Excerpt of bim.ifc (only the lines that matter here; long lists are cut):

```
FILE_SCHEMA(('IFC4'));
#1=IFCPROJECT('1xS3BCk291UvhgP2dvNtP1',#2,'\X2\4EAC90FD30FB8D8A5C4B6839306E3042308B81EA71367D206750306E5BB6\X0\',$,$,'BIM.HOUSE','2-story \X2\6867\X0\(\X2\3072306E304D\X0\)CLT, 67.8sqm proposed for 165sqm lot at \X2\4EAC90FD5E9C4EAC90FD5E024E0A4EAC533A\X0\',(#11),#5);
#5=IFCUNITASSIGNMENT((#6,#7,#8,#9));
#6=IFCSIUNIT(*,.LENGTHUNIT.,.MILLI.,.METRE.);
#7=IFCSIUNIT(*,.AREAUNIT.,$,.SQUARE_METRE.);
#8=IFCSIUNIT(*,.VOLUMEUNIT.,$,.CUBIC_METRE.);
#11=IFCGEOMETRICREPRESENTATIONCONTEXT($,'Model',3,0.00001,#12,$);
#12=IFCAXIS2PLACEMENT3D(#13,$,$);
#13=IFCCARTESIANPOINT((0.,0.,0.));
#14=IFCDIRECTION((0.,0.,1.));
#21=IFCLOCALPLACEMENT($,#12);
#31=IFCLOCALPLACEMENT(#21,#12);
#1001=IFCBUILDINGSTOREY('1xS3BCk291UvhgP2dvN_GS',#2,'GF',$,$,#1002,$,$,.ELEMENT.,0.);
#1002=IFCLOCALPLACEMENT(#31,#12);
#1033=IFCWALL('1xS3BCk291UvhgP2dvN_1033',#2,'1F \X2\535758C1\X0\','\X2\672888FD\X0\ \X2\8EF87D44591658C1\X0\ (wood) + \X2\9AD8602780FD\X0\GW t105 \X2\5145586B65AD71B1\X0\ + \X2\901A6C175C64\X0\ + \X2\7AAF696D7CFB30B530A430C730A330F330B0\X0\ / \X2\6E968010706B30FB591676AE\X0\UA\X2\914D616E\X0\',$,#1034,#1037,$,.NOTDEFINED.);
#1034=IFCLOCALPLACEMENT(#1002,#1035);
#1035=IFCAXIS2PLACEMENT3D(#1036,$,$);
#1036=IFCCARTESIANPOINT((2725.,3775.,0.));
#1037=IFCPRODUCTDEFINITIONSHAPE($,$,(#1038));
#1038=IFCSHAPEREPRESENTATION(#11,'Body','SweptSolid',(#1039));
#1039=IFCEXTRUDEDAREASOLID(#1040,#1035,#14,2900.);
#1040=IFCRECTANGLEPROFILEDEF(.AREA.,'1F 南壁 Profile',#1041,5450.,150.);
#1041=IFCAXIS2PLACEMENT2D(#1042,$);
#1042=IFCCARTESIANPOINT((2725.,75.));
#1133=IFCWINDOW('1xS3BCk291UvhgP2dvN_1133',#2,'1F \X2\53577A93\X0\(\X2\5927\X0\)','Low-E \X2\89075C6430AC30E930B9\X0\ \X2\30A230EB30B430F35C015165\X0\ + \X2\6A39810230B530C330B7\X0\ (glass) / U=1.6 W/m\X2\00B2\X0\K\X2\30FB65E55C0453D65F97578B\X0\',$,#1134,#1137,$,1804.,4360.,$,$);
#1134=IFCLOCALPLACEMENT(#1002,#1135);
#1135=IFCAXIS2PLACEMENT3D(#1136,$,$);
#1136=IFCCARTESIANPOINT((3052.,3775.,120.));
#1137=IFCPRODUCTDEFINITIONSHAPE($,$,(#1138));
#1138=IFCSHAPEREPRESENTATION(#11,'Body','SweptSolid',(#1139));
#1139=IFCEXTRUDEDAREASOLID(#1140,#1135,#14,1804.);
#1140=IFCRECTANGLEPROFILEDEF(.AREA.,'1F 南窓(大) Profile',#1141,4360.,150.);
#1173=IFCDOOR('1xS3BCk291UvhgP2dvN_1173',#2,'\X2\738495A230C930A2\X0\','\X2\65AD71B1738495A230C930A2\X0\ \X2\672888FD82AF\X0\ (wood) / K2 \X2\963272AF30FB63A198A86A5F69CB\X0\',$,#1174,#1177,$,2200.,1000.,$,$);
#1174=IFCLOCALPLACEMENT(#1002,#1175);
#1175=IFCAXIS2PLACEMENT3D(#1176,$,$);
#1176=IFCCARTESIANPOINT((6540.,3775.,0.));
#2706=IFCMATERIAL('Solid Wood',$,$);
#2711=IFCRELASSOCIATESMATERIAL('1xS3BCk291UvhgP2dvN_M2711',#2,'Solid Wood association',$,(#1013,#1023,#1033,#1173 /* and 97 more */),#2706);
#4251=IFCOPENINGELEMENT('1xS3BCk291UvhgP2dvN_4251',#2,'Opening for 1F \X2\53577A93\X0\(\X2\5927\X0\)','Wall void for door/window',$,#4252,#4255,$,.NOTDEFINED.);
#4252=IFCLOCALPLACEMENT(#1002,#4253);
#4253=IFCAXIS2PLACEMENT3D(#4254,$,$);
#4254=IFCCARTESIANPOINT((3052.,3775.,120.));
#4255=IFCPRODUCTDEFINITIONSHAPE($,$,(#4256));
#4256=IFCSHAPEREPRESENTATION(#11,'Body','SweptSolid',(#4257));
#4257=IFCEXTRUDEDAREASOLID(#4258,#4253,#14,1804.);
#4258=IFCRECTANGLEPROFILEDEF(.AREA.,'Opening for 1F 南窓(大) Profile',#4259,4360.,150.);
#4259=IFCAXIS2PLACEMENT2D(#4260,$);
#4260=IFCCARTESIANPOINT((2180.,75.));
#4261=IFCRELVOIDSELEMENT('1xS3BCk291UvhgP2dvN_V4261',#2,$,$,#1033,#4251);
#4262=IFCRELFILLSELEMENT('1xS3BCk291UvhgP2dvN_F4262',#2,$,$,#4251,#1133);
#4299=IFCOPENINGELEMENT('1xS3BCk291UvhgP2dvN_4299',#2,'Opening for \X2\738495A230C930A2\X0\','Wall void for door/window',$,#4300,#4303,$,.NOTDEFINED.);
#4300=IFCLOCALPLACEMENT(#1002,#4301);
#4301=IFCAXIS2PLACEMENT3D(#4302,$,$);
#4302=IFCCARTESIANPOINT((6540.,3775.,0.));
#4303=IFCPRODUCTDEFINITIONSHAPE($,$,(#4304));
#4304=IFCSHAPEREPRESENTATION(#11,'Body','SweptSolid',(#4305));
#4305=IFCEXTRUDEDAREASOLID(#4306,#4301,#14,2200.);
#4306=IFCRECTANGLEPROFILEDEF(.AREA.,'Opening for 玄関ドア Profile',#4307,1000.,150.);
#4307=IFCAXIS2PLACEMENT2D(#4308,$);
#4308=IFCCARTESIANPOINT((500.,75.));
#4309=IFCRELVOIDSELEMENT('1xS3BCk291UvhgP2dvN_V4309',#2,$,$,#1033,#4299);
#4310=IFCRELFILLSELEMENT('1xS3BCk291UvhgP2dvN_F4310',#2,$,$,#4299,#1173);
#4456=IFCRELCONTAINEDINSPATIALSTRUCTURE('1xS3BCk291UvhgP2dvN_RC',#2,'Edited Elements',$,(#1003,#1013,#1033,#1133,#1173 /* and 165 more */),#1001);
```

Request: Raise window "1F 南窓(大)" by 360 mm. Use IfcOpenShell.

```python
import numpy as np
import ifcopenshell
import ifcopenshell.api.geometry
import ifcopenshell.util.placement
import ifcopenshell.util.unit

model = ifcopenshell.open("bim.ifc")
unit_scale = ifcopenshell.util.unit.calculate_unit_scale(model)

window = model.by_guid("1xS3BCk291UvhgP2dvN_1133")
opening = window.FillsVoids[0].RelatingOpeningElement
dz = 360.0

shift = np.array([0.0, 0.0, dz])
# The window is not placed relative to its opening, so move both.
for product in (opening, window):
    matrix = ifcopenshell.util.placement.get_local_placement(product.ObjectPlacement)
    matrix[:3, 3] += shift
    ifcopenshell.api.geometry.edit_object_placement(model, product=product, matrix=matrix, is_si=False)

print(f"moved by {dz * unit_scale:+.3f} m")

model.write("bim_edited.ifc")
```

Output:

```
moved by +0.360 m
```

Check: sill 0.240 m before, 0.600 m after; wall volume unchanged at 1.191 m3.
